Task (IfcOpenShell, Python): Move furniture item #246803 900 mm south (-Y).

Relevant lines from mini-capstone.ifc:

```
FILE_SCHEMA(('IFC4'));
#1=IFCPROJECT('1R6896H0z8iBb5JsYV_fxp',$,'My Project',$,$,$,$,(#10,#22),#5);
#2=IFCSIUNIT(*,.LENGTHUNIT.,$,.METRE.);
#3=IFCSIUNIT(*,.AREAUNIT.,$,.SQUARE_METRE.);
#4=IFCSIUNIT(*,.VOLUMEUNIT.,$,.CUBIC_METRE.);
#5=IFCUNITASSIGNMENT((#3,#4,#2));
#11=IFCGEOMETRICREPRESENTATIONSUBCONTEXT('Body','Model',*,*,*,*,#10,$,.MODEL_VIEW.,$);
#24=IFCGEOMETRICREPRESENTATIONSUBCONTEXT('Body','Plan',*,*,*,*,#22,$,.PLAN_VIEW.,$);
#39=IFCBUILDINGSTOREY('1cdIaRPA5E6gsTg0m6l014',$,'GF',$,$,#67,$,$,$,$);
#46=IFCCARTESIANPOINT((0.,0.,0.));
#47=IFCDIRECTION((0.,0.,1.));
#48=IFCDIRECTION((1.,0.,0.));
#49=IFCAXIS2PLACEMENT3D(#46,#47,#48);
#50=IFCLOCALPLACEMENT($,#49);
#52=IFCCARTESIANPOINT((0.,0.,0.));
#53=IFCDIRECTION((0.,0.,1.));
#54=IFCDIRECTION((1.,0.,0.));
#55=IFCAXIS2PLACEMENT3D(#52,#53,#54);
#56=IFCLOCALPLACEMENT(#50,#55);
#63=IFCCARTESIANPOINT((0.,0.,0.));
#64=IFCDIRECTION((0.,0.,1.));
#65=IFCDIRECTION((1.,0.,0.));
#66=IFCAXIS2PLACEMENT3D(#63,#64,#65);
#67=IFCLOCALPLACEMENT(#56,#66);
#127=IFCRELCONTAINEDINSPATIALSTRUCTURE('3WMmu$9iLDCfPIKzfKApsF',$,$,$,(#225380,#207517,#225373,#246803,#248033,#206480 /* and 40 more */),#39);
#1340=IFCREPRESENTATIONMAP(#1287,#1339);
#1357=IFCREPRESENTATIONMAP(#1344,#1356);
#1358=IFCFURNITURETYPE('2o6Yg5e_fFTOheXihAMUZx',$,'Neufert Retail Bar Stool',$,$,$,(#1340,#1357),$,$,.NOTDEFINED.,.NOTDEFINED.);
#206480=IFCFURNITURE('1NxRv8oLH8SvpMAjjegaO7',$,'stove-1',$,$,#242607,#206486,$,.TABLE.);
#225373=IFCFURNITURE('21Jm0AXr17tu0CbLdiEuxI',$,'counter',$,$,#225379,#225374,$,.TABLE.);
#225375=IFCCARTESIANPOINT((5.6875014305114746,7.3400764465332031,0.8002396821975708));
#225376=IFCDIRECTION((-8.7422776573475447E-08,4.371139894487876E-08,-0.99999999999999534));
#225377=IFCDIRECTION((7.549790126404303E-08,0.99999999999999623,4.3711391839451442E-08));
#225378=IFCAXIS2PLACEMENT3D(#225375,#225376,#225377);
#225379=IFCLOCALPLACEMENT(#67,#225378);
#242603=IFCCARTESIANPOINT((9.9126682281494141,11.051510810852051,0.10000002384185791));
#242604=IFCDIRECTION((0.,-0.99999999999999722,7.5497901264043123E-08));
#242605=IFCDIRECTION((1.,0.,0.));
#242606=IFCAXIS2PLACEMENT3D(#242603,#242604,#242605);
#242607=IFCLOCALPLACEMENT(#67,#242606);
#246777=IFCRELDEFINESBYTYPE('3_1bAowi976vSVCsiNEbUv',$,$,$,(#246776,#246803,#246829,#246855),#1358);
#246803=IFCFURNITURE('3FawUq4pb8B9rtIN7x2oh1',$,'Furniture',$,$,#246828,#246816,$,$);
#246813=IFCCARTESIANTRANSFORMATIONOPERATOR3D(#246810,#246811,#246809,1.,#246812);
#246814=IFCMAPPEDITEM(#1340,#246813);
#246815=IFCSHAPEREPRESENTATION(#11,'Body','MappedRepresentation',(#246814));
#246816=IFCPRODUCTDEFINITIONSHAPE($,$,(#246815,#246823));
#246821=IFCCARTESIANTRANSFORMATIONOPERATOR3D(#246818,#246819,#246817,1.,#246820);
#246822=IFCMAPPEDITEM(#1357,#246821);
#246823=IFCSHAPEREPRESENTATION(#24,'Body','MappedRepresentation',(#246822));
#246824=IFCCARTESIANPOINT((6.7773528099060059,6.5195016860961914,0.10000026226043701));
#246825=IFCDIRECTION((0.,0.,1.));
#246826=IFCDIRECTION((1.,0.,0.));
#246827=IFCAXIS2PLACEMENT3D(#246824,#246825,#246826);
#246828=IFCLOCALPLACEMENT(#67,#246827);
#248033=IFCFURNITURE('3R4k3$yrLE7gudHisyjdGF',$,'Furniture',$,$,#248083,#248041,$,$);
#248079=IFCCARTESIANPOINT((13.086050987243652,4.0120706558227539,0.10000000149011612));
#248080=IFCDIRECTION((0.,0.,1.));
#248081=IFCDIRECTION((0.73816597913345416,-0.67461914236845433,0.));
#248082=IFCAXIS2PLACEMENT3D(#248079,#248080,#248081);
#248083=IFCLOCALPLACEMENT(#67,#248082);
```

```python
import ifcopenshell
import ifcopenshell.api.geometry
import ifcopenshell.util.placement

model = ifcopenshell.open("mini-capstone.ifc")

item = model.by_id(246803)
matrix = ifcopenshell.util.placement.get_local_placement(item.ObjectPlacement)
matrix[1, 3] -= 0.9
ifcopenshell.api.geometry.edit_object_placement(model, product=item, matrix=matrix, is_si=False)

print(ifcopenshell.util.placement.get_local_placement(item.ObjectPlacement).round(3) + 0.0)

model.write("mini-capstone_edited.ifc")
```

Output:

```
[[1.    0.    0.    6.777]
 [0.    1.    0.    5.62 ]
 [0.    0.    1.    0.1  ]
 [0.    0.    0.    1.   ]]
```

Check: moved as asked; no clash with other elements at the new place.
